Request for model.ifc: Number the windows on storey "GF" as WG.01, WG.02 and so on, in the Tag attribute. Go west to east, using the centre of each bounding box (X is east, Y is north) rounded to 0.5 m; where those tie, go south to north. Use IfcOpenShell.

First a look at what the model holds.

```python
import ifcopenshell
import ifcopenshell.util.element
import ifcopenshell.util.placement

model = ifcopenshell.open("model.ifc")
print(model.schema)
storey = next(s for s in model.by_type("IfcBuildingStorey") if s.Name == "GF")
windows = [e for e in ifcopenshell.util.element.get_decomposition(storey) if e.is_a("IfcWindow")]
for e in sorted(windows, key=lambda e: e.id()):
    origin = ifcopenshell.util.placement.get_local_placement(e.ObjectPlacement)[:3, 3]
    print(e.id(), e.Tag, e.Name, origin.round(2) + 0.0, sep=" | ")
```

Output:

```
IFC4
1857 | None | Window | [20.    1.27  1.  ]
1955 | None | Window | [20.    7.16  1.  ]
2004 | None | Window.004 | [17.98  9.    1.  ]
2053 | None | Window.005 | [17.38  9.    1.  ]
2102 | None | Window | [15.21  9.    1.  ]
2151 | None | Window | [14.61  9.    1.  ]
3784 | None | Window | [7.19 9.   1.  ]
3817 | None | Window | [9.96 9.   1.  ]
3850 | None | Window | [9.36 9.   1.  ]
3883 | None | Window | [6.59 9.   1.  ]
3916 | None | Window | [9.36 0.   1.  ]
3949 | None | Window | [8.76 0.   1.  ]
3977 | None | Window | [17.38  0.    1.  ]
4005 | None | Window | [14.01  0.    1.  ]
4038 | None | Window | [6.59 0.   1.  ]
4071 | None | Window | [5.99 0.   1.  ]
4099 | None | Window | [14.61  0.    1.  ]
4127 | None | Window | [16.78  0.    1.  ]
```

```python
import ifcopenshell
import ifcopenshell.geom
import ifcopenshell.util.element
import ifcopenshell.util.shape

model = ifcopenshell.open("model.ifc")
settings = ifcopenshell.geom.settings()
settings.set("use-world-coords", True)


def centre(element):
    shape = ifcopenshell.geom.create_shape(settings, element)
    return ifcopenshell.util.shape.get_bbox_centroid(shape.geometry)


storey = next(s for s in model.by_type("IfcBuildingStorey") if s.Name == "GF")
windows = [e for e in ifcopenshell.util.element.get_decomposition(storey) if e.is_a("IfcWindow")]

# Insertion points can sit at a corner or the storey origin, so sort by the geometry (in metres).
centres = {e: centre(e) for e in windows}
windows.sort(key=lambda e: (round(centres[e][0] / 0.5), centres[e][1]))

for i, e in enumerate(windows, start=1):
    number = f"WG.{i:02d}"
    e.Tag = number
    print(e.id(), number)

model.write("model_updated.ifc")
```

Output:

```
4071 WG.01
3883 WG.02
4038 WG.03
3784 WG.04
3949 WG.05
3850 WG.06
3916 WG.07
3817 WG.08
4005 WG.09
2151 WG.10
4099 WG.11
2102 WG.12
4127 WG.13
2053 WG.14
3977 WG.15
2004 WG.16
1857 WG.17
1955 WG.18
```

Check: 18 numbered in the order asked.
